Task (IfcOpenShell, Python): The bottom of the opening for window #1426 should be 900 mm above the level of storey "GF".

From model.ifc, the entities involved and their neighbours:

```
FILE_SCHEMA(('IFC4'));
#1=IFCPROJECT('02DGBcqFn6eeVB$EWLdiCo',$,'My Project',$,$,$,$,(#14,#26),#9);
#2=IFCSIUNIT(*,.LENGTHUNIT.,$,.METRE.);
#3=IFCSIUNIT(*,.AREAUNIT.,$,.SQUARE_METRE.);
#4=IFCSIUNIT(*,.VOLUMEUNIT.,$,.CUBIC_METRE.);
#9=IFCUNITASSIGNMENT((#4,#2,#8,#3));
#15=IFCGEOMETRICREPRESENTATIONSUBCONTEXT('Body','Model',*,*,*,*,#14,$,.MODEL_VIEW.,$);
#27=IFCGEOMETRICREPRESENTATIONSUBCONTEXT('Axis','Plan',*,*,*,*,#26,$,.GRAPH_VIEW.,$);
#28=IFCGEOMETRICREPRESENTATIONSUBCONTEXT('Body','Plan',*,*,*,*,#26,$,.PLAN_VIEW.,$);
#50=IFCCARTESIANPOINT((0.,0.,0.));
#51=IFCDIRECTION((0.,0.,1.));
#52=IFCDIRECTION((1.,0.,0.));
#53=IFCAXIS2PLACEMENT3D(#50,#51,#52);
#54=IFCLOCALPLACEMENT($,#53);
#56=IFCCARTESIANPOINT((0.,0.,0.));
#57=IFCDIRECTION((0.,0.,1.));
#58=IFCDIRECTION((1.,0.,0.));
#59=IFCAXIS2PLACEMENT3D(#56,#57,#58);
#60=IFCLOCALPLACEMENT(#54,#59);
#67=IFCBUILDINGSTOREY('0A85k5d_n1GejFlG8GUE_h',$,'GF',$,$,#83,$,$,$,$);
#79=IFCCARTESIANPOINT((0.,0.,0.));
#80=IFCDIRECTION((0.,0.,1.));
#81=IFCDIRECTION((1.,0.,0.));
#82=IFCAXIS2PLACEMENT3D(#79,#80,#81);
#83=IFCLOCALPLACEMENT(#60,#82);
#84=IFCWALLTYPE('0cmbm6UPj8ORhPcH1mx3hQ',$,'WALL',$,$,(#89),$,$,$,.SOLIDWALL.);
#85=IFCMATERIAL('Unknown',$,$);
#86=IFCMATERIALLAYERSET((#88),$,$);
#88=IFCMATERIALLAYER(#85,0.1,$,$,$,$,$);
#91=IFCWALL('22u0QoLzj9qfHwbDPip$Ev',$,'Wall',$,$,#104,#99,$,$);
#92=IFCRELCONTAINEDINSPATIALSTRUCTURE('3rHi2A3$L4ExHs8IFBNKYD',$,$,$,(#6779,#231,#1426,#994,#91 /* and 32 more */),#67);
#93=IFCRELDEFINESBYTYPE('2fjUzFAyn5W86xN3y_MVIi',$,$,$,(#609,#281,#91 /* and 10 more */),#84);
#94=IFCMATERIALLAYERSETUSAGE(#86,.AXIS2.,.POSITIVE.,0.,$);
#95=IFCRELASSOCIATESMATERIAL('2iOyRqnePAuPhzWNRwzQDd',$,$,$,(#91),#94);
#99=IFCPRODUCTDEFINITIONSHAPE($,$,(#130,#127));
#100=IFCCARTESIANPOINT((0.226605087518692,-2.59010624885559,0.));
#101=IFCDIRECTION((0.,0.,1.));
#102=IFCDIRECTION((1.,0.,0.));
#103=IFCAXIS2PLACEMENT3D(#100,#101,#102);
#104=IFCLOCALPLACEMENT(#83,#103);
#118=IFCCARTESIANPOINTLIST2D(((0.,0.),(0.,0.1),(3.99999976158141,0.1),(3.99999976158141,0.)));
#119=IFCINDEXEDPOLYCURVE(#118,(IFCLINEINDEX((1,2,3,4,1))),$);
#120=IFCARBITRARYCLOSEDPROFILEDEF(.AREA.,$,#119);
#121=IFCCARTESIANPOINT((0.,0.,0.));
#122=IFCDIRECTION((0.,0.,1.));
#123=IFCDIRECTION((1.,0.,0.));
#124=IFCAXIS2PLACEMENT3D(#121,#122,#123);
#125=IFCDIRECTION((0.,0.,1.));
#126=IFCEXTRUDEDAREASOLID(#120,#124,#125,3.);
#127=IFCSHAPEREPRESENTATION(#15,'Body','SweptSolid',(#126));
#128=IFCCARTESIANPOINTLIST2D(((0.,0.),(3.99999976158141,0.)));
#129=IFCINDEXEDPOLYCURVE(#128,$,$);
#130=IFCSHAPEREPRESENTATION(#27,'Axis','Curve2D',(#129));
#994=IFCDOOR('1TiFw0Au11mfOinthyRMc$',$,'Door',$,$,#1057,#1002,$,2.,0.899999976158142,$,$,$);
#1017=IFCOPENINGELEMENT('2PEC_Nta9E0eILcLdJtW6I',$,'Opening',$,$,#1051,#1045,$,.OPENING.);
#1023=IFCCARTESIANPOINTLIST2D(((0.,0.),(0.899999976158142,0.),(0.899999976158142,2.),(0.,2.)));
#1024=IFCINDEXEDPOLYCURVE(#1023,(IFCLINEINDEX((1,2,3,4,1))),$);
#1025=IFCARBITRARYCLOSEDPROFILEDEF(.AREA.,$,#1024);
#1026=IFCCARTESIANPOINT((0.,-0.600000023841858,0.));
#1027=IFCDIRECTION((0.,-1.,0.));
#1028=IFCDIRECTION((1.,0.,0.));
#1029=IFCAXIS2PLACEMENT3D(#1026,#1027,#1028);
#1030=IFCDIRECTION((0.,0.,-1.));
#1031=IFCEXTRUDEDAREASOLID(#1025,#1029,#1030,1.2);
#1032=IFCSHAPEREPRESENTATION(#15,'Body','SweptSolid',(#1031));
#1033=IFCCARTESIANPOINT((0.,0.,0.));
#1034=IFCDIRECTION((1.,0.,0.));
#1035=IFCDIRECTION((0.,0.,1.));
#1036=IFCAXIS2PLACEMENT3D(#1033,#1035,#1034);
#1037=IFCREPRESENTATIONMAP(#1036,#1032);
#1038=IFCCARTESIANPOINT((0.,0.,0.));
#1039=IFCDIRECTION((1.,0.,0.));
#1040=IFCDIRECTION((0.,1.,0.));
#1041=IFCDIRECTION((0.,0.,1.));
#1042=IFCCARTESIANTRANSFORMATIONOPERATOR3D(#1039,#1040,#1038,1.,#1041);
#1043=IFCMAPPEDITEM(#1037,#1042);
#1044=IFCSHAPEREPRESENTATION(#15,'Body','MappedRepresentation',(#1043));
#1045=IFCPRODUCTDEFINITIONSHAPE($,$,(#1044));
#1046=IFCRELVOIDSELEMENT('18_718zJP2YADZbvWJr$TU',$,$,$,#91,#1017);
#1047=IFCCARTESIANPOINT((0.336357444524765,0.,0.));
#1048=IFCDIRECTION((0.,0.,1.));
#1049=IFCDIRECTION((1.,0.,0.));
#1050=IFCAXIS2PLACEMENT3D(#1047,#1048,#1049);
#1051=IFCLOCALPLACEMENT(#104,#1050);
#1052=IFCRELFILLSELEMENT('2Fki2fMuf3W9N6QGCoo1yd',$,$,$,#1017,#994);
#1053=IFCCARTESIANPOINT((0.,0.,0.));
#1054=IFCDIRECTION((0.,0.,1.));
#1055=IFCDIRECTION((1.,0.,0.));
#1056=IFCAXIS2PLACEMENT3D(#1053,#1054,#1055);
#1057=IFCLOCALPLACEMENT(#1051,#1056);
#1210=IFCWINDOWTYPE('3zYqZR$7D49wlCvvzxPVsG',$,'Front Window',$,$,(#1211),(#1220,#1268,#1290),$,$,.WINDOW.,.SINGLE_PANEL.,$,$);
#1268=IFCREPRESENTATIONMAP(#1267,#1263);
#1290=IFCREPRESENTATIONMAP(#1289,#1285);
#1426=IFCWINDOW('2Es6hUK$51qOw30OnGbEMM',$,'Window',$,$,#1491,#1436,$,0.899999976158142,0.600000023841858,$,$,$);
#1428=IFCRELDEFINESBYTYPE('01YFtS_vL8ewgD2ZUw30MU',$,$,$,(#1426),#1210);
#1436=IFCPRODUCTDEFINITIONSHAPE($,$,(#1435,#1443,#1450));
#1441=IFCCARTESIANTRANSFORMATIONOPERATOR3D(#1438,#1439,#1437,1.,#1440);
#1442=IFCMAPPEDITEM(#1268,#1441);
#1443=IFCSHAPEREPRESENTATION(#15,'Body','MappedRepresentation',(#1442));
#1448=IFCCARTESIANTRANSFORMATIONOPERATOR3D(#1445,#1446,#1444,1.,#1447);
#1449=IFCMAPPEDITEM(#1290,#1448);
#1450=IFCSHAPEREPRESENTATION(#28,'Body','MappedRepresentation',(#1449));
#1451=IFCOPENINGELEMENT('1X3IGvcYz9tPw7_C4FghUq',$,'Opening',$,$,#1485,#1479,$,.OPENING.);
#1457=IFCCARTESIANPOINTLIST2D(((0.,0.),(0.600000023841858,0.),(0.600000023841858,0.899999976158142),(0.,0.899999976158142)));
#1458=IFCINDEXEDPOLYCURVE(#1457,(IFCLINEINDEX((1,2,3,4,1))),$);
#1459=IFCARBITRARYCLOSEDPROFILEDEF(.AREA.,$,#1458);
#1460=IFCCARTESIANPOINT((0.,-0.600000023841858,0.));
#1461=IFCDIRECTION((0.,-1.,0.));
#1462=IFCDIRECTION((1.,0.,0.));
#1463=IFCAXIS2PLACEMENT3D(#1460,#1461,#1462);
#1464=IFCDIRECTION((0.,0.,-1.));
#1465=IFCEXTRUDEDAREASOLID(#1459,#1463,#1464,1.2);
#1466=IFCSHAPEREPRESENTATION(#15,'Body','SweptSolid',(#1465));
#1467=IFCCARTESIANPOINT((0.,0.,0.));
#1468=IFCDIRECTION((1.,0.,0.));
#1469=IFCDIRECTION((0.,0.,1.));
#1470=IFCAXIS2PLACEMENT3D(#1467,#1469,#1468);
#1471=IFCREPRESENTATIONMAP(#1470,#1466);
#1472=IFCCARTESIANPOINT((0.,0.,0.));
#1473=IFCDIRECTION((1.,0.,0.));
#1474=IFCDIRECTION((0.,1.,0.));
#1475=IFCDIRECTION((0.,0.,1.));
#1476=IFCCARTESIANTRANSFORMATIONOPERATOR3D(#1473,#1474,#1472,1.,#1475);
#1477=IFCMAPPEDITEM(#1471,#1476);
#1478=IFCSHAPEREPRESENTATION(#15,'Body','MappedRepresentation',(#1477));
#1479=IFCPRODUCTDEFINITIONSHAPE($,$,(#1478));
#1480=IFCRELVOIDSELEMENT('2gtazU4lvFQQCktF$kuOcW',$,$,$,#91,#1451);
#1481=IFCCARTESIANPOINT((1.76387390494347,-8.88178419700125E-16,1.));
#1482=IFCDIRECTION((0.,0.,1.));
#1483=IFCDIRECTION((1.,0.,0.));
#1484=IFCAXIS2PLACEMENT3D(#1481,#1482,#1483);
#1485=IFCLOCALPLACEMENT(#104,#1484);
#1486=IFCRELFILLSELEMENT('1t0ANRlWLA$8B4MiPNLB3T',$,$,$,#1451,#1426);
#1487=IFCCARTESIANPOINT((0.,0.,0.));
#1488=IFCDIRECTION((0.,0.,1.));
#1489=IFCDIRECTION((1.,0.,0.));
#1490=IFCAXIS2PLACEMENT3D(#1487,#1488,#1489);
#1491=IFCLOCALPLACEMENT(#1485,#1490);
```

```python
import numpy as np
import ifcopenshell
import ifcopenshell.api.geometry
import ifcopenshell.geom
import ifcopenshell.util.element
import ifcopenshell.util.placement
import ifcopenshell.util.shape
import ifcopenshell.util.unit

model = ifcopenshell.open("model.ifc")
unit_scale = ifcopenshell.util.unit.calculate_unit_scale(model)

window = model.by_guid("2Es6hUK$51qOw30OnGbEMM")
opening = window.FillsVoids[0].RelatingOpeningElement
storey = ifcopenshell.util.element.get_container(window, ifc_class="IfcBuildingStorey")
level = ifcopenshell.util.placement.get_local_placement(storey.ObjectPlacement)[2, 3]

# The opening's origin need not be at the sill, so measure its lowest point.
shape = ifcopenshell.geom.create_shape(ifcopenshell.geom.settings(), opening)
bottom = ifcopenshell.util.shape.get_shape_bottom_elevation(shape, shape.geometry) / unit_scale
dz = level + 0.9 - bottom

shift = np.array([0.0, 0.0, dz])
# The window is placed relative to its opening, so it follows when the opening moves.
matrix = ifcopenshell.util.placement.get_local_placement(opening.ObjectPlacement)
matrix[:3, 3] += shift
ifcopenshell.api.geometry.edit_object_placement(
    model, product=opening, matrix=matrix, is_si=False, should_transform_children=True
)

print(f"moved by {dz * unit_scale:+.3f} m")

model.write("model_edited.ifc")
```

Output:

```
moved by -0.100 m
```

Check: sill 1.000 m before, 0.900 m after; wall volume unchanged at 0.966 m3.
